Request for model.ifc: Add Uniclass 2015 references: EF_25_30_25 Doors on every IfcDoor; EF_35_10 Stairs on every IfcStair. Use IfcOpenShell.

First a look at what the model holds.

```python
import ifcopenshell

model = ifcopenshell.open("model.ifc")
print(model.schema)
print("classifications:", [c.Name for c in model.by_type("IfcClassification")])
for ifc_class in ("IfcDoor", "IfcRoof", "IfcStair", "IfcWall", "IfcWindow"):
    print(ifc_class, len(model.by_type(ifc_class)))
```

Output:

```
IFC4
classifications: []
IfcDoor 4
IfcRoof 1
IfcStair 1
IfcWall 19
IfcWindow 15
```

```python
import ifcopenshell
import ifcopenshell.api.classification

model = ifcopenshell.open("model.ifc")

system = ifcopenshell.api.classification.add_classification(model, classification="Uniclass 2015")

codes = {
    "IfcDoor": ("EF_25_30_25", "Doors"),
    "IfcStair": ("EF_35_10", "Stairs"),
}
for ifc_class, (code, name) in codes.items():
    products = model.by_type(ifc_class)
    ifcopenshell.api.classification.add_reference(
        model, products=products, classification=system, identification=code, name=name
    )
    print(code, len(products))

model.write("model_rev.ifc")
```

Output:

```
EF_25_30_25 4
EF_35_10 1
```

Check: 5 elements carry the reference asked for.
